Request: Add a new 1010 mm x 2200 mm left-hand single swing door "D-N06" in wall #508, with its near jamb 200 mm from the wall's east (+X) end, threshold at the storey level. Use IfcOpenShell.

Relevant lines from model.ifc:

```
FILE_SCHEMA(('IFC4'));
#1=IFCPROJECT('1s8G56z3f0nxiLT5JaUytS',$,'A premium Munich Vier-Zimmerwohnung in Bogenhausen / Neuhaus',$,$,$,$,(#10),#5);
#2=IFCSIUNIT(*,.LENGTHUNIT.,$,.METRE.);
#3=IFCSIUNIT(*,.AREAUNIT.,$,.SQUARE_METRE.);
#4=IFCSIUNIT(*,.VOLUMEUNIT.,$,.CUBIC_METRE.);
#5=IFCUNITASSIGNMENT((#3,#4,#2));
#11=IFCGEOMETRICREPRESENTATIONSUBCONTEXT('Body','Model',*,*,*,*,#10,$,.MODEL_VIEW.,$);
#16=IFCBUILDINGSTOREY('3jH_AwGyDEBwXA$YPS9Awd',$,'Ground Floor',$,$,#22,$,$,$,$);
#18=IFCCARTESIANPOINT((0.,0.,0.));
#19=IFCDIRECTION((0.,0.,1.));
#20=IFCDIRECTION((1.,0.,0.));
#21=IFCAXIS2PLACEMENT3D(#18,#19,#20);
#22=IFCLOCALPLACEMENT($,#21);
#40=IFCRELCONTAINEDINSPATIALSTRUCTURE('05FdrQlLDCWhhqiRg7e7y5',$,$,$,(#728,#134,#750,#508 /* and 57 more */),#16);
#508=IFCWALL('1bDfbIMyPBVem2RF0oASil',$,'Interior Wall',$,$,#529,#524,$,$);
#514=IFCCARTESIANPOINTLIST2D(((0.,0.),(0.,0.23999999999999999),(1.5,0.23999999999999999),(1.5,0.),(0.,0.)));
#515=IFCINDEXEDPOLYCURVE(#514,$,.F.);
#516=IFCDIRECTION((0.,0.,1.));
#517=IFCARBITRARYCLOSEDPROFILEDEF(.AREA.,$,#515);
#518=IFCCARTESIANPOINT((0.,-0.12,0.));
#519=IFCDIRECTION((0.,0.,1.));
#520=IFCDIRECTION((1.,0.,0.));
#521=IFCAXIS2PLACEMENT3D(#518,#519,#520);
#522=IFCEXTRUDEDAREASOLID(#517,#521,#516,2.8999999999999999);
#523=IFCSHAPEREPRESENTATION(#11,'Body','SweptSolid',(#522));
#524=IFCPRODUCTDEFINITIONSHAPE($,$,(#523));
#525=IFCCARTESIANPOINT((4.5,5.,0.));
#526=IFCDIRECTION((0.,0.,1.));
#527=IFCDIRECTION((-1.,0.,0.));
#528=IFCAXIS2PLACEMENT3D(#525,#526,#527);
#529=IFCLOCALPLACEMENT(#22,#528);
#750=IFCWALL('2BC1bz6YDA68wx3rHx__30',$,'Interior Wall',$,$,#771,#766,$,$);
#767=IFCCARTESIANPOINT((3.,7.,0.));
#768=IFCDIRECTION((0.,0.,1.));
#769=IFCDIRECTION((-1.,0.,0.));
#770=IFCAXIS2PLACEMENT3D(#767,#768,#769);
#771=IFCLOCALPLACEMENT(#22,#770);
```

```python
import numpy as np
import ifcopenshell
import ifcopenshell.api.feature
import ifcopenshell.api.geometry
import ifcopenshell.api.root
import ifcopenshell.api.spatial
import ifcopenshell.geom
import ifcopenshell.util.element
import ifcopenshell.util.placement
import ifcopenshell.util.representation
import ifcopenshell.util.shape
import ifcopenshell.util.unit

model = ifcopenshell.open("model.ifc")
unit_scale = ifcopenshell.util.unit.calculate_unit_scale(model)
settings = ifcopenshell.geom.settings()


def volume(element):
    """Net volume in cubic metres, openings subtracted."""
    shape = ifcopenshell.geom.create_shape(settings, element)
    return ifcopenshell.util.shape.get_volume(shape.geometry)


wall = model.by_id(508)
storey = ifcopenshell.util.element.get_container(wall, ifc_class="IfcBuildingStorey")
context = ifcopenshell.util.representation.get_context(model, "Model", "Body", "MODEL_VIEW")
before = volume(wall)

width, height, from_end, sill = 1.01, 2.2, 0.2, 0.0  # metres

# The wall runs along its own X axis, and the end named is its -X end.
wall_shape = ifcopenshell.geom.create_shape(settings, wall)
x, y, z = ifcopenshell.util.shape.get_vertices(wall_shape.geometry).T
start = x.min() + from_end
face, thickness = float(y.min()), float(y.max() - y.min())
wall_matrix = ifcopenshell.util.placement.get_local_placement(wall.ObjectPlacement)
level = ifcopenshell.util.placement.get_local_placement(storey.ObjectPlacement)[2, 3]


def in_wall(x, y):
    """Placement at x, y metres in the wall's axes, at sill height."""
    matrix = wall_matrix.copy()
    matrix[:, 3] = wall_matrix @ np.array([x / unit_scale, y / unit_scale, 0.0, 1.0])
    matrix[2, 3] = level + sill / unit_scale
    return matrix


# Opening: a box that overshoots both wall faces by 50 mm.
opening = ifcopenshell.api.root.create_entity(model, ifc_class="IfcOpeningElement", predefined_type="OPENING")
box = ifcopenshell.api.geometry.add_wall_representation(
    model, context=context, length=width, height=height, thickness=thickness + 0.1
)
ifcopenshell.api.geometry.assign_representation(model, product=opening, representation=box)
ifcopenshell.api.geometry.edit_object_placement(model, product=opening, matrix=in_wall(start, face - 0.05), is_si=False)
ifcopenshell.api.feature.add_feature(model, feature=opening, element=wall)

door = ifcopenshell.api.root.create_entity(model, ifc_class="IfcDoor", name="D-N06", predefined_type="DOOR")
door.OverallWidth, door.OverallHeight = width / unit_scale, height / unit_scale
door.OperationType = "SINGLE_SWING_LEFT"
body = ifcopenshell.api.geometry.add_door_representation(
    model,
    context=context,
    overall_width=door.OverallWidth,
    overall_height=door.OverallHeight,
    operation_type="SINGLE_SWING_LEFT",
    lining_properties={"LiningDepth": thickness / unit_scale, "ThresholdDepth": thickness / unit_scale},
)
ifcopenshell.api.geometry.assign_representation(model, product=door, representation=body)
ifcopenshell.api.spatial.assign_container(model, products=[door], relating_structure=storey)
ifcopenshell.api.feature.add_filling(model, opening=opening, element=door)

# The lining spans the wall, so the door starts at the wall face.
ifcopenshell.api.geometry.edit_object_placement(model, product=door, matrix=in_wall(start, face), is_si=False)

after = volume(wall)

print(f"wall volume {before:.3f} -> {after:.3f} m3")

model.write("model_rev.ifc")
```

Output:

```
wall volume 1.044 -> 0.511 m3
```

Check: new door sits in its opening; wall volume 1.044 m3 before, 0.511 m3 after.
